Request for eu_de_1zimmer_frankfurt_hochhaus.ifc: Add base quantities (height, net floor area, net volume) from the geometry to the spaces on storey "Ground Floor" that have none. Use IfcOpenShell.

First a look at what the model holds.

```python
import ifcopenshell
import ifcopenshell.util.element
import ifcopenshell.util.unit

model = ifcopenshell.open("eu_de_1zimmer_frankfurt_hochhaus.ifc")
print(model.schema)
for unit_type in ("LENGTHUNIT", "AREAUNIT", "VOLUMEUNIT"):
    print(unit_type, ifcopenshell.util.unit.calculate_unit_scale(model, unit_type))
storey = next(s for s in model.by_type("IfcBuildingStorey") if s.Name == "Ground Floor")
spaces = [e for e in ifcopenshell.util.element.get_decomposition(storey) if e.is_a("IfcSpace")]
for e in sorted(spaces, key=lambda e: e.id()):
    print(e.id(), e.is_a(), e.Name, list(ifcopenshell.util.element.get_psets(e, qtos_only=True)), sep=" | ")
```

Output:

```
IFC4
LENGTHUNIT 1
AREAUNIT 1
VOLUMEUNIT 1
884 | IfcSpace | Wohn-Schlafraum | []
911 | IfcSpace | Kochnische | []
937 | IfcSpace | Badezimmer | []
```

```python
import ifcopenshell
import ifcopenshell.api.pset
import ifcopenshell.geom
import ifcopenshell.util.element
import ifcopenshell.util.shape
import ifcopenshell.util.unit

model = ifcopenshell.open("eu_de_1zimmer_frankfurt_hochhaus.ifc")
unit_scale = ifcopenshell.util.unit.calculate_unit_scale(model)
area_scale = ifcopenshell.util.unit.calculate_unit_scale(model, "AREAUNIT")
volume_scale = ifcopenshell.util.unit.calculate_unit_scale(model, "VOLUMEUNIT")
settings = ifcopenshell.geom.settings()

storey = next(s for s in model.by_type("IfcBuildingStorey") if s.Name == "Ground Floor")
spaces = [e for e in ifcopenshell.util.element.get_decomposition(storey) if e.is_a("IfcSpace")]

for e in sorted(spaces, key=lambda e: e.id()):
    if ifcopenshell.util.element.get_psets(e, qtos_only=True, should_inherit=False):
        continue
    # Geometry comes back in metres, in the element's own axes.
    shape = ifcopenshell.geom.create_shape(settings, e)
    values = {
        "Height": ifcopenshell.util.shape.get_z(shape.geometry) / unit_scale,
        "NetFloorArea": ifcopenshell.util.shape.get_footprint_area(shape.geometry) / area_scale,
        "NetVolume": ifcopenshell.util.shape.get_volume(shape.geometry) / volume_scale,
    }
    qto = ifcopenshell.api.pset.add_qto(model, product=e, name="Qto_SpaceBaseQuantities")
    ifcopenshell.api.pset.edit_qto(model, qto=qto, properties=values)
    print(e.id(), {k: round(v, 3) for k, v in values.items()})

model.write("eu_de_1zimmer_frankfurt_hochhaus_updated.ifc")
```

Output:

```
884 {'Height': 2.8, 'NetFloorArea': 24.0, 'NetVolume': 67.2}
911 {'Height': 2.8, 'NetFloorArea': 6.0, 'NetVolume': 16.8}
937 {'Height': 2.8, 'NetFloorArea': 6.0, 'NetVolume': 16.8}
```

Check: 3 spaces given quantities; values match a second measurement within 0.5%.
